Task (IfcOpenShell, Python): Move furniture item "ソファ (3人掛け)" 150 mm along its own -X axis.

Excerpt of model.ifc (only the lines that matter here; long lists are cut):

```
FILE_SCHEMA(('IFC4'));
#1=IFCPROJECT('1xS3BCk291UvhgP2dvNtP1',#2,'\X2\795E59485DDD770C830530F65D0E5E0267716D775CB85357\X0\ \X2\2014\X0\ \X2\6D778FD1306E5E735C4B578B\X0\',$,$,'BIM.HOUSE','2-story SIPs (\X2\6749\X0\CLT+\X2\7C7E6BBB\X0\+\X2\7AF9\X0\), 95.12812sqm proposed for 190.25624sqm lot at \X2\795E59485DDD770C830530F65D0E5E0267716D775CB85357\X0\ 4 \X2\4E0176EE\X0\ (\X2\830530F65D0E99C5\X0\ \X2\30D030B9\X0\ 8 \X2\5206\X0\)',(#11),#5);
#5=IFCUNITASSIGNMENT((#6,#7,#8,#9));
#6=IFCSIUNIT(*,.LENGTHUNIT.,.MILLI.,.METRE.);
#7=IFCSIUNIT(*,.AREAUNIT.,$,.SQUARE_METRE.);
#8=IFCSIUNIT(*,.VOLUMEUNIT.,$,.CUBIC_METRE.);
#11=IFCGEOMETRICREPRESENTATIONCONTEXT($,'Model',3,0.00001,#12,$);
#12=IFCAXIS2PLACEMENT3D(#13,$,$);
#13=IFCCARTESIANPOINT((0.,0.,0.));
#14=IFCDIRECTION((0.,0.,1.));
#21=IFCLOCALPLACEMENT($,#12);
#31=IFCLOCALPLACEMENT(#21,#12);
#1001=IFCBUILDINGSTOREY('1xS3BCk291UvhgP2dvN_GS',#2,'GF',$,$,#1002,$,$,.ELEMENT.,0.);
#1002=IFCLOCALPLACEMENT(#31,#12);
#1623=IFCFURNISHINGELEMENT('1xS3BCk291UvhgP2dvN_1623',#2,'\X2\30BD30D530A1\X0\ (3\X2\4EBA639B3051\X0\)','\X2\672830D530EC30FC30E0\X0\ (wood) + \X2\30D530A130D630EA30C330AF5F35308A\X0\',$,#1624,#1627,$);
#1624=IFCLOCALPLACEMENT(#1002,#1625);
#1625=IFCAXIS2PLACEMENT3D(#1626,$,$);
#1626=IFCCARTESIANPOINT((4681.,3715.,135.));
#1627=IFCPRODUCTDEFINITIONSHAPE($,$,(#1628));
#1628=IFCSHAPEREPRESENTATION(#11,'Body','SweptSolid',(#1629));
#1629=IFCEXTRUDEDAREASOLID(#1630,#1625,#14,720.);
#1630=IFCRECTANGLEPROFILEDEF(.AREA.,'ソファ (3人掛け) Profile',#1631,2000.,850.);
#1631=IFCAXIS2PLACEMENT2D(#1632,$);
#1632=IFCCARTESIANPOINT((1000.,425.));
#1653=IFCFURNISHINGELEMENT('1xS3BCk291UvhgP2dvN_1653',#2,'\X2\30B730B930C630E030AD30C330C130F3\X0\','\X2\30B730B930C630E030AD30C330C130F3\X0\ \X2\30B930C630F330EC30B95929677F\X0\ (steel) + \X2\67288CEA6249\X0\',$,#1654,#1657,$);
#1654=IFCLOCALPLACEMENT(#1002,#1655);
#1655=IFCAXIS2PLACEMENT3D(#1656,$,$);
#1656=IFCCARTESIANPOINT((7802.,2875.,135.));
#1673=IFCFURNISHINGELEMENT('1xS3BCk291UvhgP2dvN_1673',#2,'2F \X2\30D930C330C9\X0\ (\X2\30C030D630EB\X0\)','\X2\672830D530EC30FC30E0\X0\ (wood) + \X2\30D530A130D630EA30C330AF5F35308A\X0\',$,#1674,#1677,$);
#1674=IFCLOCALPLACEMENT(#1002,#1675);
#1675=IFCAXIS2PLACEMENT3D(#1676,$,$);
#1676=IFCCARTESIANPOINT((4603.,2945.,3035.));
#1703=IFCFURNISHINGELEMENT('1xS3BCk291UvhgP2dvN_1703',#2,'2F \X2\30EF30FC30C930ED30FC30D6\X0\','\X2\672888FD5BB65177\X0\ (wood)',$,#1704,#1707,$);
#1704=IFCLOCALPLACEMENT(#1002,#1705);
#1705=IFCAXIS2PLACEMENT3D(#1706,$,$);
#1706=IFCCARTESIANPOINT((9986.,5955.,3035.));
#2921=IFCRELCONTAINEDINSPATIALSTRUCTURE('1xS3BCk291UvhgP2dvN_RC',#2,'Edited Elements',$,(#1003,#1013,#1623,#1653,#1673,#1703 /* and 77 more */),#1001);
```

```python
import ifcopenshell
import ifcopenshell.api.geometry
import ifcopenshell.util.placement
import ifcopenshell.util.unit

model = ifcopenshell.open("model.ifc")
unit_scale = ifcopenshell.util.unit.calculate_unit_scale(model)

item = model.by_guid("1xS3BCk291UvhgP2dvN_1623")
matrix = ifcopenshell.util.placement.get_local_placement(item.ObjectPlacement)
matrix[:3, 3] -= matrix[:3, 0] * 0.15 / unit_scale
ifcopenshell.api.geometry.edit_object_placement(model, product=item, matrix=matrix, is_si=False)

print(ifcopenshell.util.placement.get_local_placement(item.ObjectPlacement).round(3) + 0.0)

model.write("model-out.ifc")
```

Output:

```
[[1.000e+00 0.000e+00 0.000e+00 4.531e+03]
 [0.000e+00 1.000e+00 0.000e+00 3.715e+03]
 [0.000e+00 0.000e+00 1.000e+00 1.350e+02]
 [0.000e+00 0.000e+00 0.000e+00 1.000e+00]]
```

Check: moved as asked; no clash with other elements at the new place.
